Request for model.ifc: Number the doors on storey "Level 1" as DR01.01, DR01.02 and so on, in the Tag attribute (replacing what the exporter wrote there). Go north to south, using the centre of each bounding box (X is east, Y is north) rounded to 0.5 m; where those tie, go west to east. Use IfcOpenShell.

First a look at what the model holds.

```python
import ifcopenshell
import ifcopenshell.util.element
import ifcopenshell.util.placement

model = ifcopenshell.open("model.ifc")
print(model.schema)
storey = next(s for s in model.by_type("IfcBuildingStorey") if s.Name == "Level 1")
doors = [e for e in ifcopenshell.util.element.get_decomposition(storey) if e.is_a("IfcDoor")]
for e in sorted(doors, key=lambda e: e.id()):
    origin = ifcopenshell.util.placement.get_local_placement(e.ObjectPlacement)[:3, 3]
    print(e.id(), e.Tag, e.Name, origin.round(2) + 0.0, sep=" | ")
```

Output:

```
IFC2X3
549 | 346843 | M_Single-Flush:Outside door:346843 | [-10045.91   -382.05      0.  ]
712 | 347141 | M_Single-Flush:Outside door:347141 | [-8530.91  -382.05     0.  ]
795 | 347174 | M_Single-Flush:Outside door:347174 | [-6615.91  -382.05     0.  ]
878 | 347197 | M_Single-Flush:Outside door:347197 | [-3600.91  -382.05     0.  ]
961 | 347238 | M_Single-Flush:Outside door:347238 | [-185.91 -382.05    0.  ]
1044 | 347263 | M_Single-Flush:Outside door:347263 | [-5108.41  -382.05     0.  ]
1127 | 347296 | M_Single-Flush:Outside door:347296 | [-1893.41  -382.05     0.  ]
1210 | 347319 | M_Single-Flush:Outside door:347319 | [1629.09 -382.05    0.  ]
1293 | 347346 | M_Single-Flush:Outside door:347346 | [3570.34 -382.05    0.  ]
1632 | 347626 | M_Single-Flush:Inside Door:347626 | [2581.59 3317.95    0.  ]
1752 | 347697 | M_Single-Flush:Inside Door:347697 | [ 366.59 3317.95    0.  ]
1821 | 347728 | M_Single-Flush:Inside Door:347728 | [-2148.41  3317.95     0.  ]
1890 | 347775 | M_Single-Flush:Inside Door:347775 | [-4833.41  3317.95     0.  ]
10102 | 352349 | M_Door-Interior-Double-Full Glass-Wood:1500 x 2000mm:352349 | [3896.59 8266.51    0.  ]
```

```python
import ifcopenshell
import ifcopenshell.geom
import ifcopenshell.util.element
import ifcopenshell.util.shape

model = ifcopenshell.open("model.ifc")
settings = ifcopenshell.geom.settings()
settings.set("use-world-coords", True)


def centre(element):
    shape = ifcopenshell.geom.create_shape(settings, element)
    return ifcopenshell.util.shape.get_bbox_centroid(shape.geometry)


storey = next(s for s in model.by_type("IfcBuildingStorey") if s.Name == "Level 1")
doors = [e for e in ifcopenshell.util.element.get_decomposition(storey) if e.is_a("IfcDoor")]

# Insertion points can sit at a corner or the storey origin, so sort by the geometry (in metres).
centres = {e: centre(e) for e in doors}
doors.sort(key=lambda e: (-round(centres[e][1] / 0.5), centres[e][0]))

for i, e in enumerate(doors, start=1):
    number = f"DR01.{i:02d}"
    e.Tag = number
    print(e.id(), number)

model.write("model_rev.ifc")
```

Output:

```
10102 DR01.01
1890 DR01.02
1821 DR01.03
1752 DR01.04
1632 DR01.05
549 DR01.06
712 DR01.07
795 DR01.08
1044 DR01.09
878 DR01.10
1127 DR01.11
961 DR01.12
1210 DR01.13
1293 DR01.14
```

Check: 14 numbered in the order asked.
